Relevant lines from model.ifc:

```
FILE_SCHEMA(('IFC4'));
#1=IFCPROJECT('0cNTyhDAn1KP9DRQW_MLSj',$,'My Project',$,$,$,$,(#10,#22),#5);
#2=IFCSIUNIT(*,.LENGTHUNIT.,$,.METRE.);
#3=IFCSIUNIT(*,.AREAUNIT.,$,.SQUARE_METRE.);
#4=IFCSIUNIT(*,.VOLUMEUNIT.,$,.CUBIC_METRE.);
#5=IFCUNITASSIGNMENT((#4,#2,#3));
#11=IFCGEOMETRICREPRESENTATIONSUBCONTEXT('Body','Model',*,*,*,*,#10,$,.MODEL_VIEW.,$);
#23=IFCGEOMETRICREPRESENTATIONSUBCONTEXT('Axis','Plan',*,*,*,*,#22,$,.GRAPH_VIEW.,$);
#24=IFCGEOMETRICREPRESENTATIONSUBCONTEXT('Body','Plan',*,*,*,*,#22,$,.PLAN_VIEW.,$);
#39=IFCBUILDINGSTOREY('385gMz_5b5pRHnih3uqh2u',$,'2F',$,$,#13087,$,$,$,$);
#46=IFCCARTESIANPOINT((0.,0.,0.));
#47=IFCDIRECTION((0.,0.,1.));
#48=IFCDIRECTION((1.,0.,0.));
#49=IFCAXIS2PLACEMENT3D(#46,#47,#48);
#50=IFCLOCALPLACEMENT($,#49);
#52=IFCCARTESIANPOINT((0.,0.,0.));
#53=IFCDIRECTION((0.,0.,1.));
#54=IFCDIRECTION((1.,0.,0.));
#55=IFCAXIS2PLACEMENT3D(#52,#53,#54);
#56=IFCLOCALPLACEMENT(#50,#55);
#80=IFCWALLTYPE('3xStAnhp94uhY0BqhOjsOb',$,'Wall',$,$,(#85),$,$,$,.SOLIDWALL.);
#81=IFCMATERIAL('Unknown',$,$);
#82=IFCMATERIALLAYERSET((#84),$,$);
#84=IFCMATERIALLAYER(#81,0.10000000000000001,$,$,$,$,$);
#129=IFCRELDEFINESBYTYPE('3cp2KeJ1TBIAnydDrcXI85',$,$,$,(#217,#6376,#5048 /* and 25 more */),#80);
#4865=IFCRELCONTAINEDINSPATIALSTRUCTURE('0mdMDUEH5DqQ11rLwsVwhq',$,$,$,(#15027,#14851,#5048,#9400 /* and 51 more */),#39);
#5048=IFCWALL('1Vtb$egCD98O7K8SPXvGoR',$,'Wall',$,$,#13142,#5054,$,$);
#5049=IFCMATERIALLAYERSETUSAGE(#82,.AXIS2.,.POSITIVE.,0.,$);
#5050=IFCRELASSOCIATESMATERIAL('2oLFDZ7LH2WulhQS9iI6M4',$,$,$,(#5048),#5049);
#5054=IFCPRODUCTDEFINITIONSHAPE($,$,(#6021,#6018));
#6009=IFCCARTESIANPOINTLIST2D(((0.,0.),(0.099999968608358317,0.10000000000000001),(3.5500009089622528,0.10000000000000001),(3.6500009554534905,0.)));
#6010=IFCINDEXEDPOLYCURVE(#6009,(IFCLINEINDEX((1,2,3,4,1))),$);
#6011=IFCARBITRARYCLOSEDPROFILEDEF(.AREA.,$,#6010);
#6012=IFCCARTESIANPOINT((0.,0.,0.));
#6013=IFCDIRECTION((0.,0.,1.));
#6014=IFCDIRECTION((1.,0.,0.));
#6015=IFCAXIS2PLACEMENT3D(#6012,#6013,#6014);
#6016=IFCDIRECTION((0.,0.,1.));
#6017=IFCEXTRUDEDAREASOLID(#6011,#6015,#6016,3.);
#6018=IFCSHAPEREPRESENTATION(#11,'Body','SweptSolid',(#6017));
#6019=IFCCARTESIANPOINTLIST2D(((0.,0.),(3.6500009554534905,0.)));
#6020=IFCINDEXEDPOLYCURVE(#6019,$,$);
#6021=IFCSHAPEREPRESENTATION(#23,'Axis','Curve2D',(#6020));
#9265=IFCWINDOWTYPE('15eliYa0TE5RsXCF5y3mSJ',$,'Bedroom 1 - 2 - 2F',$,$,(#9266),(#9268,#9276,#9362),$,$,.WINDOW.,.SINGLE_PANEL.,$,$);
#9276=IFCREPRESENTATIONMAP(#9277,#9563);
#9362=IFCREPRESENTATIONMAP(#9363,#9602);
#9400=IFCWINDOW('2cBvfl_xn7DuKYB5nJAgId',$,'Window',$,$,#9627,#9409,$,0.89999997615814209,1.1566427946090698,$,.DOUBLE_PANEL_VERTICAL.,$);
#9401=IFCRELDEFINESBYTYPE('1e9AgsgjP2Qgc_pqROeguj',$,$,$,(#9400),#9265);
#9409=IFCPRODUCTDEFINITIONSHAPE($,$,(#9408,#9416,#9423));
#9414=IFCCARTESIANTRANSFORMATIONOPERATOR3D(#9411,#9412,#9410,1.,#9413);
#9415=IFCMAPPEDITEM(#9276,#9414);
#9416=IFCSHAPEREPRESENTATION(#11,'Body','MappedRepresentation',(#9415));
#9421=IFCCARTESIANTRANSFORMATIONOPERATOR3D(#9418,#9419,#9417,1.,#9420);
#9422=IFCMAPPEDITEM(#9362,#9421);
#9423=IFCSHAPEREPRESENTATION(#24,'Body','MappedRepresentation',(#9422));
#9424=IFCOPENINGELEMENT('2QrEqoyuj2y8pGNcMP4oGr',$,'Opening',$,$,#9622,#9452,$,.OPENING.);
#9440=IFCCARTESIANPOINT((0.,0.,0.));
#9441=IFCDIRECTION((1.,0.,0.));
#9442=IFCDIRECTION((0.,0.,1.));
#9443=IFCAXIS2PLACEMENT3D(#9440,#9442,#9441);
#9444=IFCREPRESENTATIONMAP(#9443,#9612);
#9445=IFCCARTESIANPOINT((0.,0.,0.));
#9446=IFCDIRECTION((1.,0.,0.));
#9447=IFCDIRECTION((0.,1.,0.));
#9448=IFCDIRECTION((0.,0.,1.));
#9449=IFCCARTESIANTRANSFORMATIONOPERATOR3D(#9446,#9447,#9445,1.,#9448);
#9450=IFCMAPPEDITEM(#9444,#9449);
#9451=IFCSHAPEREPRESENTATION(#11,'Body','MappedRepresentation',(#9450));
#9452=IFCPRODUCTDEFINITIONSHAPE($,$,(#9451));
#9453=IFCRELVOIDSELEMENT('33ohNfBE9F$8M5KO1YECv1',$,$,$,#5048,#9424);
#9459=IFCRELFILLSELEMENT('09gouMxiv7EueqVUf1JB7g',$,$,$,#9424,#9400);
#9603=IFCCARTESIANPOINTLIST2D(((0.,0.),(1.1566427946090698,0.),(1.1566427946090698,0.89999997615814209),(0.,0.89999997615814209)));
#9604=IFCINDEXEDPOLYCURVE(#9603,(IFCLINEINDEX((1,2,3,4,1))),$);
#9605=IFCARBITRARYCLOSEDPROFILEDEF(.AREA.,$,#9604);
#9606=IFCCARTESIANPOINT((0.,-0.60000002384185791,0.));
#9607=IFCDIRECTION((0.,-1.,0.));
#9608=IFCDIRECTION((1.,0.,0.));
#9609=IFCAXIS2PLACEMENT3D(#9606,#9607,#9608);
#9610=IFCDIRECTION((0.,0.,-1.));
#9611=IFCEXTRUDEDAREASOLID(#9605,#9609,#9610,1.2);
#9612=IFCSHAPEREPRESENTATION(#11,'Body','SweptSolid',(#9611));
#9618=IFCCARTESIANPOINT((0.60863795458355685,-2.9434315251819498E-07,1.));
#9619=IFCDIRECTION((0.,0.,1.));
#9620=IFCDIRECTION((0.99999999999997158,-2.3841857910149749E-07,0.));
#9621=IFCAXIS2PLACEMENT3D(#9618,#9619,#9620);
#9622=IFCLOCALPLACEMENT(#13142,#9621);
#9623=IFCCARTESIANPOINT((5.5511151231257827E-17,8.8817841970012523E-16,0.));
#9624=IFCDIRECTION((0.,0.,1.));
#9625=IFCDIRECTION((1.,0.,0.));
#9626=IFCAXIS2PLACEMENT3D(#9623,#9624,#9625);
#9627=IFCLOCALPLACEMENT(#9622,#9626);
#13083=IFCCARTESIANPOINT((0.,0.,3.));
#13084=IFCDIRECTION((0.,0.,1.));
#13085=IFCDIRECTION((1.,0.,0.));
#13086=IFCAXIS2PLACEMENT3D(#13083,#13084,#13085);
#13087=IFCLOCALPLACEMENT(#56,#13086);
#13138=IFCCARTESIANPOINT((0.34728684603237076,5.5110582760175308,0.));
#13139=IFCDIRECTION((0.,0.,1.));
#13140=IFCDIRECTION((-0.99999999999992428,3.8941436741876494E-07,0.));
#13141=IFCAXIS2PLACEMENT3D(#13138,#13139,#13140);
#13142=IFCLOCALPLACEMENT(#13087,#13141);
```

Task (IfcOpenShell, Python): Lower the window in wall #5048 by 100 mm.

```python
import numpy as np
import ifcopenshell
import ifcopenshell.api.geometry
import ifcopenshell.util.placement
import ifcopenshell.util.unit

model = ifcopenshell.open("model.ifc")
unit_scale = ifcopenshell.util.unit.calculate_unit_scale(model)

window = model.by_guid("2cBvfl_xn7DuKYB5nJAgId")
opening = window.FillsVoids[0].RelatingOpeningElement
dz = -0.1 / unit_scale

shift = np.array([0.0, 0.0, dz])
# The window is placed relative to its opening, so it follows when the opening moves.
matrix = ifcopenshell.util.placement.get_local_placement(opening.ObjectPlacement)
matrix[:3, 3] += shift
ifcopenshell.api.geometry.edit_object_placement(
    model, product=opening, matrix=matrix, is_si=False, should_transform_children=True
)

print(f"moved by {dz * unit_scale:+.3f} m")

model.write("model_edited.ifc")
```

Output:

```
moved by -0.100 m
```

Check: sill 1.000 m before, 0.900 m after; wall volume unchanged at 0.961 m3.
